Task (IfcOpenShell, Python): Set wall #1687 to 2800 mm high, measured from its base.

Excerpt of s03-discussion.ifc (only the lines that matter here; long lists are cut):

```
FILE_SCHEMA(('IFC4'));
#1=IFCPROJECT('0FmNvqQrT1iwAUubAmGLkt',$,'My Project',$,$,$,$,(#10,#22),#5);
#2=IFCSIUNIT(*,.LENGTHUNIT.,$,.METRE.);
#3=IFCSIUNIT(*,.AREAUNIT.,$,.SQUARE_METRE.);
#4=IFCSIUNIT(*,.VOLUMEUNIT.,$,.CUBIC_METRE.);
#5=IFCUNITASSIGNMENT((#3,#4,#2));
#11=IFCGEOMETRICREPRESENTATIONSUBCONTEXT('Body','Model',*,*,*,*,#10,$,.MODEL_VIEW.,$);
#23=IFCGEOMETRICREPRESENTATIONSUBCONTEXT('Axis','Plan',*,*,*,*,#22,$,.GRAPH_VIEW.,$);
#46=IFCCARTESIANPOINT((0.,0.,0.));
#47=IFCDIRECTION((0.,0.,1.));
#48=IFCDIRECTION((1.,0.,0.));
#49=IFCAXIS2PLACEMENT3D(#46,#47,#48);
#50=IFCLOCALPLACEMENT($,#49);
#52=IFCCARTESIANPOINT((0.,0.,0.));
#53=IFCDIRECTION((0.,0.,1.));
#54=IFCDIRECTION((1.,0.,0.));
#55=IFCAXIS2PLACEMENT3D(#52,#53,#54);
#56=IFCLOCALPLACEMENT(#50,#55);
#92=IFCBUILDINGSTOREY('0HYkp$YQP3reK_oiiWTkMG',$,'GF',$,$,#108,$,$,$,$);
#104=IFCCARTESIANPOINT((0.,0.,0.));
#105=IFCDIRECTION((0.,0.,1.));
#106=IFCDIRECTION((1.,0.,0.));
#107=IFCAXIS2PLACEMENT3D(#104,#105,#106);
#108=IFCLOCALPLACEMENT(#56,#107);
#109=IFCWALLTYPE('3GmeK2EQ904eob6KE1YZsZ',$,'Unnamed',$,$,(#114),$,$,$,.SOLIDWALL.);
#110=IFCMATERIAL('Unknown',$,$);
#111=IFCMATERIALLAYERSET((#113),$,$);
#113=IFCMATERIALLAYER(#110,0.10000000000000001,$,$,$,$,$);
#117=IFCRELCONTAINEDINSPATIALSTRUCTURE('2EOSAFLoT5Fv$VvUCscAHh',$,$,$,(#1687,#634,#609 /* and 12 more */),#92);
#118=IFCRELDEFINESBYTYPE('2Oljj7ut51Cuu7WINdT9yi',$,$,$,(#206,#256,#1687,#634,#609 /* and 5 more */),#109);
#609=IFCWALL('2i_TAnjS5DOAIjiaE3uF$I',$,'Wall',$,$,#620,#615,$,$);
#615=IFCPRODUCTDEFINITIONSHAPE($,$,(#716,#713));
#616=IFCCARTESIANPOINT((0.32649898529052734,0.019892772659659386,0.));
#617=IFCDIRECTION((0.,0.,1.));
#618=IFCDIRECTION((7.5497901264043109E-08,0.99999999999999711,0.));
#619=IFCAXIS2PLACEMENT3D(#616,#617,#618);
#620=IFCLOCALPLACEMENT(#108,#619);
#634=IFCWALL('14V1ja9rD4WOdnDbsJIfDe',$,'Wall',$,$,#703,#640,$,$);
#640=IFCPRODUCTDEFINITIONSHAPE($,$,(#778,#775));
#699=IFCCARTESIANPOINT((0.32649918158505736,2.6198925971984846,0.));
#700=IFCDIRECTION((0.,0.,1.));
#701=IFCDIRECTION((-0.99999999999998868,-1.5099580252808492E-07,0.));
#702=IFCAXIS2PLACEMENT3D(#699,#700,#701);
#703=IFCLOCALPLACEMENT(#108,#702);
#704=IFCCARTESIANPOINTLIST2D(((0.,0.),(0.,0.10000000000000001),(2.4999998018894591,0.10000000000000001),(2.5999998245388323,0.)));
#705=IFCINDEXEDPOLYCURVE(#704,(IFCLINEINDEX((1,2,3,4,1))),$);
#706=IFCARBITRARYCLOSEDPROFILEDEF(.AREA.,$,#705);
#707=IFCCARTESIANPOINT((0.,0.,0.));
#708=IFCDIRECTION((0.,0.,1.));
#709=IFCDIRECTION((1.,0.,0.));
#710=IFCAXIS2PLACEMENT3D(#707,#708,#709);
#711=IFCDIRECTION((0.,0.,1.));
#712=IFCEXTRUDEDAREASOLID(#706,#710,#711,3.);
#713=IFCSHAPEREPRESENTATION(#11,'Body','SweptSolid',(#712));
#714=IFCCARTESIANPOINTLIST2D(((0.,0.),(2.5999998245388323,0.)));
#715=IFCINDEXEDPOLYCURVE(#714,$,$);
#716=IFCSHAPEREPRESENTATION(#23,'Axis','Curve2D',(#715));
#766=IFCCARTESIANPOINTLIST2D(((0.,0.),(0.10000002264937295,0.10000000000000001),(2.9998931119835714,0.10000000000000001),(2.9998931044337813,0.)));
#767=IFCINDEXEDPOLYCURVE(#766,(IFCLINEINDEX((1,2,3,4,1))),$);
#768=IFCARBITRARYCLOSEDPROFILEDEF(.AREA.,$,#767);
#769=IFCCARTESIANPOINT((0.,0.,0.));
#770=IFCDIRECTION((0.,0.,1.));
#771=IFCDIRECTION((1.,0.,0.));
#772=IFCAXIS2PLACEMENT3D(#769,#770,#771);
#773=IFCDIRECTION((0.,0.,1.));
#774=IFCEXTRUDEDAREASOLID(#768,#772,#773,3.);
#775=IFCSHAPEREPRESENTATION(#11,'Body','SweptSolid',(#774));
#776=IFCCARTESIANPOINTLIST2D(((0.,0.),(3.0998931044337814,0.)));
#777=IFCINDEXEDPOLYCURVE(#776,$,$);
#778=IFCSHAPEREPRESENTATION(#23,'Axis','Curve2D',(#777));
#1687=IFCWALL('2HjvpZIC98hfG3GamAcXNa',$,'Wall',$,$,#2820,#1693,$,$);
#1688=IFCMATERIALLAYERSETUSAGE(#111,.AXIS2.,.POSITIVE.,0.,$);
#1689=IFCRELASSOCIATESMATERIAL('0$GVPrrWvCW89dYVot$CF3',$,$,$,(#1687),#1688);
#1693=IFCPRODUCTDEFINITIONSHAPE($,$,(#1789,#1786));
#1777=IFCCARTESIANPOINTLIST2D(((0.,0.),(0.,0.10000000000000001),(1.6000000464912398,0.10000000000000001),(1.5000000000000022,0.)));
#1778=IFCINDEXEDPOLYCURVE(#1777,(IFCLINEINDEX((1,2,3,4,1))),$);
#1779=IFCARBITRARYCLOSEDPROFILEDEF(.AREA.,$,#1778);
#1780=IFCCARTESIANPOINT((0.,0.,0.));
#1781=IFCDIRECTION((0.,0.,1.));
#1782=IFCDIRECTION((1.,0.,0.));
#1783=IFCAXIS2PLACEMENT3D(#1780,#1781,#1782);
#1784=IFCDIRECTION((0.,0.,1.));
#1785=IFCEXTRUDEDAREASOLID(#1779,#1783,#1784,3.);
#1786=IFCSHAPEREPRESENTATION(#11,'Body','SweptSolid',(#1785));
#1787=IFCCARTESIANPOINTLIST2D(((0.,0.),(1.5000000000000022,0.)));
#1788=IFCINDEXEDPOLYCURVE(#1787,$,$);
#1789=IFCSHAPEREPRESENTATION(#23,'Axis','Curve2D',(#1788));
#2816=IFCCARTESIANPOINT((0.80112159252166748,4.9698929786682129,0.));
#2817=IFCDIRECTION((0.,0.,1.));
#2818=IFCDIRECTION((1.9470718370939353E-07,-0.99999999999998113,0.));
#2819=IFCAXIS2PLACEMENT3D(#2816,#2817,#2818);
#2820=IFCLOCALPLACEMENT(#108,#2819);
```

```python
import ifcopenshell
import ifcopenshell.geom
import ifcopenshell.util.representation
import ifcopenshell.util.shape
import ifcopenshell.util.unit

model = ifcopenshell.open("s03-discussion.ifc")
unit_scale = ifcopenshell.util.unit.calculate_unit_scale(model)
settings = ifcopenshell.geom.settings()


def volume(element):
    """Net volume in cubic metres, openings subtracted."""
    shape = ifcopenshell.geom.create_shape(settings, element)
    return ifcopenshell.util.shape.get_volume(shape.geometry)


wall = model.by_guid("2HjvpZIC98hfG3GamAcXNa")
before = volume(wall)

body = ifcopenshell.util.representation.get_representation(wall, "Model", "Body")
solid = body.Items[0]
old_height = solid.Depth
solid.Depth = 2.8 / unit_scale
after = volume(wall)

print(f"height {old_height:g} -> {solid.Depth:g}, volume {before:.3f} -> {after:.3f} m3")

model.write("s03-discussion_updated.ifc")
```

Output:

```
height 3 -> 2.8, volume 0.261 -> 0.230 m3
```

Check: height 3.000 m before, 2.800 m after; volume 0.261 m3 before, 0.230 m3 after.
